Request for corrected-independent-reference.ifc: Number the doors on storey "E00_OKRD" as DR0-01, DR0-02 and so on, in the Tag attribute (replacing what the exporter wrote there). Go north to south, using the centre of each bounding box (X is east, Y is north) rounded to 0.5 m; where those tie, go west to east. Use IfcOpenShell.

First a look at what the model holds.

```python
import ifcopenshell
import ifcopenshell.util.element
import ifcopenshell.util.placement

model = ifcopenshell.open("corrected-independent-reference.ifc")
print(model.schema)
storey = next(s for s in model.by_type("IfcBuildingStorey") if s.Name == "E00_OKRD")
doors = [e for e in ifcopenshell.util.element.get_decomposition(storey) if e.is_a("IfcDoor")]
for e in sorted(doors, key=lambda e: e.id()):
    origin = ifcopenshell.util.placement.get_local_placement(e.ObjectPlacement)[:3, 3]
    print(e.id(), e.Tag, e.Name, origin.round(2) + 0.0, sep=" | ")
```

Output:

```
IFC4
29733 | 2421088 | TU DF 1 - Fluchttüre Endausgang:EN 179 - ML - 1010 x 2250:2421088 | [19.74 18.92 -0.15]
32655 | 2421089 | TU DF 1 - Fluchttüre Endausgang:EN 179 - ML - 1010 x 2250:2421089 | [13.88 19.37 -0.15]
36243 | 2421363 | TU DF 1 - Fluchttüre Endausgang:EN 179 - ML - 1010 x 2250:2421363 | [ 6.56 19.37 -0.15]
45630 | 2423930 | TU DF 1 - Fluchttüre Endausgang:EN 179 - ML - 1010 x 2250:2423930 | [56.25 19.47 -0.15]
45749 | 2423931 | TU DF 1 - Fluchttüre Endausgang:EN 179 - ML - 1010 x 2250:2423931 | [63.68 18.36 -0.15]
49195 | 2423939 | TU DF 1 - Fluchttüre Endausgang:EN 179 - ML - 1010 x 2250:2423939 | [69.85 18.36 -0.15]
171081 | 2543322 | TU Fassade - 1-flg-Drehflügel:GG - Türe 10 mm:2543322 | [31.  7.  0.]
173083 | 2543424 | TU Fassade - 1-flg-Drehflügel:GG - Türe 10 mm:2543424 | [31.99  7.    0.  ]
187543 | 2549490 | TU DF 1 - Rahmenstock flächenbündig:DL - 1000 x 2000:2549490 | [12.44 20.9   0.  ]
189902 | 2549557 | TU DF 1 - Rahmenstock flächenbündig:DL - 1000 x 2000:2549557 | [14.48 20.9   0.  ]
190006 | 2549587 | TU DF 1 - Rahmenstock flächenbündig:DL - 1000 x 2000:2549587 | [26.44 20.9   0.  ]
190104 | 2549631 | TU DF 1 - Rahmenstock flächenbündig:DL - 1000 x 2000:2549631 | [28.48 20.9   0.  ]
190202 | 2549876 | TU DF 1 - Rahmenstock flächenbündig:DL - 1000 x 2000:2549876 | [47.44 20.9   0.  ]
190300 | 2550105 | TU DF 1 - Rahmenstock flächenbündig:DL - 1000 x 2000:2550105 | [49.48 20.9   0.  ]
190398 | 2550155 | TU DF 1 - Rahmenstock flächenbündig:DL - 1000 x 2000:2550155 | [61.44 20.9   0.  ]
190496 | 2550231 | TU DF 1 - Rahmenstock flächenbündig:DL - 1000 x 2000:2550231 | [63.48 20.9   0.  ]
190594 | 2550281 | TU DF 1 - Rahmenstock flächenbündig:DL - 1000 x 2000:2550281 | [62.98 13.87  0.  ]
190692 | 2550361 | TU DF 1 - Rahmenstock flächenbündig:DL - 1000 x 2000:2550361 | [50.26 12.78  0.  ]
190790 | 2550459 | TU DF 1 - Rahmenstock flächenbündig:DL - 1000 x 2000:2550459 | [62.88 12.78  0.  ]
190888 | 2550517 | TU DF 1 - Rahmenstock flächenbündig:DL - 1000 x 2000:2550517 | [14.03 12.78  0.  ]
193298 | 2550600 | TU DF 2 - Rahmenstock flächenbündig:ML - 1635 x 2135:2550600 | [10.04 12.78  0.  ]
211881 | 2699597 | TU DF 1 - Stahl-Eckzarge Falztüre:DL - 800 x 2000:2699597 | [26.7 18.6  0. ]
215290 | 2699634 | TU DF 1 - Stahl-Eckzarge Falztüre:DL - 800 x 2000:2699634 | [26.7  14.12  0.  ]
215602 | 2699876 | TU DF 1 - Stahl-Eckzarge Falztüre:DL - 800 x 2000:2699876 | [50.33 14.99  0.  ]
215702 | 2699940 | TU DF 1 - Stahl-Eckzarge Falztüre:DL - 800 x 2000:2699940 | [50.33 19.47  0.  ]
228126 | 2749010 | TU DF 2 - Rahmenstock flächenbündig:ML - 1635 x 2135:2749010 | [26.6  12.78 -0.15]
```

```python
import ifcopenshell
import ifcopenshell.geom
import ifcopenshell.util.element
import ifcopenshell.util.shape

model = ifcopenshell.open("corrected-independent-reference.ifc")
settings = ifcopenshell.geom.settings()
settings.set("use-world-coords", True)


def centre(element):
    shape = ifcopenshell.geom.create_shape(settings, element)
    return ifcopenshell.util.shape.get_bbox_centroid(shape.geometry)


storey = next(s for s in model.by_type("IfcBuildingStorey") if s.Name == "E00_OKRD")
doors = [e for e in ifcopenshell.util.element.get_decomposition(storey) if e.is_a("IfcDoor")]

# Insertion points can sit at a corner or the storey origin, so sort by the geometry (in metres).
centres = {e: centre(e) for e in doors}
doors.sort(key=lambda e: (-round(centres[e][1] / 0.5), centres[e][0]))

for i, e in enumerate(doors, start=1):
    number = f"DR0-{i:02d}"
    e.Tag = number
    print(e.id(), number)

model.write("corrected-independent-reference_edited.ifc")
```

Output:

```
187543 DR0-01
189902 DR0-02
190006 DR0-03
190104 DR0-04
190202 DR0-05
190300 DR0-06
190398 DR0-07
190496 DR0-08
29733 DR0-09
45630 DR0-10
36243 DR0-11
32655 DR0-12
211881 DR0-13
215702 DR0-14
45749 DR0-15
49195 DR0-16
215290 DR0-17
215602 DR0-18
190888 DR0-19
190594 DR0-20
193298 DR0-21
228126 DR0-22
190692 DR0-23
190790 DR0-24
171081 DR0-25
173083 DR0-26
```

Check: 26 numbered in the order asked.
